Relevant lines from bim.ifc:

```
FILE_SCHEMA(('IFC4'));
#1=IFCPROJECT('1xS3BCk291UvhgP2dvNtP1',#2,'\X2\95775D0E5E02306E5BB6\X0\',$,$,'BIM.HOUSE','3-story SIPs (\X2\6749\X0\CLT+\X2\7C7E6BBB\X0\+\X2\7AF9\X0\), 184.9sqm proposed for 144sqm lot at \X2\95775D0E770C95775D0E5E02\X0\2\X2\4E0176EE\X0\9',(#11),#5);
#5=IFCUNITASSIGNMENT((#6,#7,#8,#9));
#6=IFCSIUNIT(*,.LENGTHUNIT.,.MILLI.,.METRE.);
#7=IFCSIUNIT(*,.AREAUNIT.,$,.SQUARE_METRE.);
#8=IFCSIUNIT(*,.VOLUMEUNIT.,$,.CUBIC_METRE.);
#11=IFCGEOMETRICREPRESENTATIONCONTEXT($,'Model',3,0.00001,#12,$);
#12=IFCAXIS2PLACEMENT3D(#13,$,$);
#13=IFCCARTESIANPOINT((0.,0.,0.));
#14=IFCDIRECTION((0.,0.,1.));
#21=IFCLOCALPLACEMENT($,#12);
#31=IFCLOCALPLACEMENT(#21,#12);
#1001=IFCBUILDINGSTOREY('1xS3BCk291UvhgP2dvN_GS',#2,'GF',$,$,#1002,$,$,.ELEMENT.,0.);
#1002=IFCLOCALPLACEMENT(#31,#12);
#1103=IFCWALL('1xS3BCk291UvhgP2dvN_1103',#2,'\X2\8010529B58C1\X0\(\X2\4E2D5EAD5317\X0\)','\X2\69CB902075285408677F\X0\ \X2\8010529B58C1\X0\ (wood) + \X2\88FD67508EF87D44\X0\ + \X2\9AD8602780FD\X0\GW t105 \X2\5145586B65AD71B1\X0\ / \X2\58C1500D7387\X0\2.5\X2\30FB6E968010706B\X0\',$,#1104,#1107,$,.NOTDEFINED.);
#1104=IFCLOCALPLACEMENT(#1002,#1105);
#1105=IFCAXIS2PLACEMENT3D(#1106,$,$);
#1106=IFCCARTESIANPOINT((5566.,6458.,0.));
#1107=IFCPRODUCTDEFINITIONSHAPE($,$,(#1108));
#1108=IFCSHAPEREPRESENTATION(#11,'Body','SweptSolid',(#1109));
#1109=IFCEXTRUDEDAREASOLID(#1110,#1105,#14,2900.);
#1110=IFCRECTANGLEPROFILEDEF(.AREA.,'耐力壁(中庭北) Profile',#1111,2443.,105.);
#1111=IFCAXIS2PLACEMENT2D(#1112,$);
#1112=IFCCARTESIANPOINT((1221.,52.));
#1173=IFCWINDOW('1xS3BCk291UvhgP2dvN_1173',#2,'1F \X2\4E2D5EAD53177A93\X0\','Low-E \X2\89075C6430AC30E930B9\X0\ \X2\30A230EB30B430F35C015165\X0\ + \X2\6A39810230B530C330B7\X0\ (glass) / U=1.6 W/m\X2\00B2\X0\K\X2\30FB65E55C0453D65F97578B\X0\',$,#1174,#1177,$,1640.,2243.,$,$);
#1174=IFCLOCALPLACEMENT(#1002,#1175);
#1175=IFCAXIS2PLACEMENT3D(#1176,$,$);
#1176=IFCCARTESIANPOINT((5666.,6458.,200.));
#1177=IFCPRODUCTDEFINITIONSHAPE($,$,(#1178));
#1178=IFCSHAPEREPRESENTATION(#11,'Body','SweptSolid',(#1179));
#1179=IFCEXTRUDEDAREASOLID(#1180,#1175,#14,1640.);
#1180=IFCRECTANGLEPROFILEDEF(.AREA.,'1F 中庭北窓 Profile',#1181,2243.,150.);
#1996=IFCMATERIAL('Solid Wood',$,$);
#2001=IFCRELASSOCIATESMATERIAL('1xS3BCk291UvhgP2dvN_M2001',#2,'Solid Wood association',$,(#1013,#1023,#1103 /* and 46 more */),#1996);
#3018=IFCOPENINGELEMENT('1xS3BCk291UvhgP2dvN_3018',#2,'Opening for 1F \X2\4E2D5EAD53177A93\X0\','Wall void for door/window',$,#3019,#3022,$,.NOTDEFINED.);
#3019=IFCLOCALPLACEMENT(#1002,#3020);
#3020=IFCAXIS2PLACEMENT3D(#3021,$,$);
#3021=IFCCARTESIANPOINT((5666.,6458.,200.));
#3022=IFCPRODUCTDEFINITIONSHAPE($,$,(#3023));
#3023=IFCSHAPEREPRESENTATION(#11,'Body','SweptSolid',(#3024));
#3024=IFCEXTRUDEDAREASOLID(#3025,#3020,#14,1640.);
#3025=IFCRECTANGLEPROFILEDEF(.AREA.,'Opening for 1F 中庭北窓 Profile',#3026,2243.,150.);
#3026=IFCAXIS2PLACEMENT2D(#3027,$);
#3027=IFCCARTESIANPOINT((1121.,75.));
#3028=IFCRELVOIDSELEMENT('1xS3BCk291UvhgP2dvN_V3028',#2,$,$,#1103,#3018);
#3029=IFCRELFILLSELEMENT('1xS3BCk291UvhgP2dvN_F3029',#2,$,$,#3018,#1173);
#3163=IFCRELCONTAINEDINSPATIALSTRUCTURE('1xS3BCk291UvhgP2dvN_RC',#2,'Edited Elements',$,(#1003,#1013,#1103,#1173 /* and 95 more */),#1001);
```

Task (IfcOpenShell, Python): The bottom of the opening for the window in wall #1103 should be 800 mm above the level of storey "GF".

```python
import numpy as np
import ifcopenshell
import ifcopenshell.api.geometry
import ifcopenshell.geom
import ifcopenshell.util.element
import ifcopenshell.util.placement
import ifcopenshell.util.shape
import ifcopenshell.util.unit

model = ifcopenshell.open("bim.ifc")
unit_scale = ifcopenshell.util.unit.calculate_unit_scale(model)

window = model.by_guid("1xS3BCk291UvhgP2dvN_1173")
opening = window.FillsVoids[0].RelatingOpeningElement
storey = ifcopenshell.util.element.get_container(window, ifc_class="IfcBuildingStorey")
level = ifcopenshell.util.placement.get_local_placement(storey.ObjectPlacement)[2, 3]

# The opening's origin need not be at the sill, so measure its lowest point.
shape = ifcopenshell.geom.create_shape(ifcopenshell.geom.settings(), opening)
bottom = ifcopenshell.util.shape.get_shape_bottom_elevation(shape, shape.geometry) / unit_scale
dz = level + 800.0 - bottom

shift = np.array([0.0, 0.0, dz])
# The window is not placed relative to its opening, so move both.
for product in (opening, window):
    matrix = ifcopenshell.util.placement.get_local_placement(product.ObjectPlacement)
    matrix[:3, 3] += shift
    ifcopenshell.api.geometry.edit_object_placement(model, product=product, matrix=matrix, is_si=False)

print(f"moved by {dz * unit_scale:+.3f} m")

model.write("bim_v2.ifc")
```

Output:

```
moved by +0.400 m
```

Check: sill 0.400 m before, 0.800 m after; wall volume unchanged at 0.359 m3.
